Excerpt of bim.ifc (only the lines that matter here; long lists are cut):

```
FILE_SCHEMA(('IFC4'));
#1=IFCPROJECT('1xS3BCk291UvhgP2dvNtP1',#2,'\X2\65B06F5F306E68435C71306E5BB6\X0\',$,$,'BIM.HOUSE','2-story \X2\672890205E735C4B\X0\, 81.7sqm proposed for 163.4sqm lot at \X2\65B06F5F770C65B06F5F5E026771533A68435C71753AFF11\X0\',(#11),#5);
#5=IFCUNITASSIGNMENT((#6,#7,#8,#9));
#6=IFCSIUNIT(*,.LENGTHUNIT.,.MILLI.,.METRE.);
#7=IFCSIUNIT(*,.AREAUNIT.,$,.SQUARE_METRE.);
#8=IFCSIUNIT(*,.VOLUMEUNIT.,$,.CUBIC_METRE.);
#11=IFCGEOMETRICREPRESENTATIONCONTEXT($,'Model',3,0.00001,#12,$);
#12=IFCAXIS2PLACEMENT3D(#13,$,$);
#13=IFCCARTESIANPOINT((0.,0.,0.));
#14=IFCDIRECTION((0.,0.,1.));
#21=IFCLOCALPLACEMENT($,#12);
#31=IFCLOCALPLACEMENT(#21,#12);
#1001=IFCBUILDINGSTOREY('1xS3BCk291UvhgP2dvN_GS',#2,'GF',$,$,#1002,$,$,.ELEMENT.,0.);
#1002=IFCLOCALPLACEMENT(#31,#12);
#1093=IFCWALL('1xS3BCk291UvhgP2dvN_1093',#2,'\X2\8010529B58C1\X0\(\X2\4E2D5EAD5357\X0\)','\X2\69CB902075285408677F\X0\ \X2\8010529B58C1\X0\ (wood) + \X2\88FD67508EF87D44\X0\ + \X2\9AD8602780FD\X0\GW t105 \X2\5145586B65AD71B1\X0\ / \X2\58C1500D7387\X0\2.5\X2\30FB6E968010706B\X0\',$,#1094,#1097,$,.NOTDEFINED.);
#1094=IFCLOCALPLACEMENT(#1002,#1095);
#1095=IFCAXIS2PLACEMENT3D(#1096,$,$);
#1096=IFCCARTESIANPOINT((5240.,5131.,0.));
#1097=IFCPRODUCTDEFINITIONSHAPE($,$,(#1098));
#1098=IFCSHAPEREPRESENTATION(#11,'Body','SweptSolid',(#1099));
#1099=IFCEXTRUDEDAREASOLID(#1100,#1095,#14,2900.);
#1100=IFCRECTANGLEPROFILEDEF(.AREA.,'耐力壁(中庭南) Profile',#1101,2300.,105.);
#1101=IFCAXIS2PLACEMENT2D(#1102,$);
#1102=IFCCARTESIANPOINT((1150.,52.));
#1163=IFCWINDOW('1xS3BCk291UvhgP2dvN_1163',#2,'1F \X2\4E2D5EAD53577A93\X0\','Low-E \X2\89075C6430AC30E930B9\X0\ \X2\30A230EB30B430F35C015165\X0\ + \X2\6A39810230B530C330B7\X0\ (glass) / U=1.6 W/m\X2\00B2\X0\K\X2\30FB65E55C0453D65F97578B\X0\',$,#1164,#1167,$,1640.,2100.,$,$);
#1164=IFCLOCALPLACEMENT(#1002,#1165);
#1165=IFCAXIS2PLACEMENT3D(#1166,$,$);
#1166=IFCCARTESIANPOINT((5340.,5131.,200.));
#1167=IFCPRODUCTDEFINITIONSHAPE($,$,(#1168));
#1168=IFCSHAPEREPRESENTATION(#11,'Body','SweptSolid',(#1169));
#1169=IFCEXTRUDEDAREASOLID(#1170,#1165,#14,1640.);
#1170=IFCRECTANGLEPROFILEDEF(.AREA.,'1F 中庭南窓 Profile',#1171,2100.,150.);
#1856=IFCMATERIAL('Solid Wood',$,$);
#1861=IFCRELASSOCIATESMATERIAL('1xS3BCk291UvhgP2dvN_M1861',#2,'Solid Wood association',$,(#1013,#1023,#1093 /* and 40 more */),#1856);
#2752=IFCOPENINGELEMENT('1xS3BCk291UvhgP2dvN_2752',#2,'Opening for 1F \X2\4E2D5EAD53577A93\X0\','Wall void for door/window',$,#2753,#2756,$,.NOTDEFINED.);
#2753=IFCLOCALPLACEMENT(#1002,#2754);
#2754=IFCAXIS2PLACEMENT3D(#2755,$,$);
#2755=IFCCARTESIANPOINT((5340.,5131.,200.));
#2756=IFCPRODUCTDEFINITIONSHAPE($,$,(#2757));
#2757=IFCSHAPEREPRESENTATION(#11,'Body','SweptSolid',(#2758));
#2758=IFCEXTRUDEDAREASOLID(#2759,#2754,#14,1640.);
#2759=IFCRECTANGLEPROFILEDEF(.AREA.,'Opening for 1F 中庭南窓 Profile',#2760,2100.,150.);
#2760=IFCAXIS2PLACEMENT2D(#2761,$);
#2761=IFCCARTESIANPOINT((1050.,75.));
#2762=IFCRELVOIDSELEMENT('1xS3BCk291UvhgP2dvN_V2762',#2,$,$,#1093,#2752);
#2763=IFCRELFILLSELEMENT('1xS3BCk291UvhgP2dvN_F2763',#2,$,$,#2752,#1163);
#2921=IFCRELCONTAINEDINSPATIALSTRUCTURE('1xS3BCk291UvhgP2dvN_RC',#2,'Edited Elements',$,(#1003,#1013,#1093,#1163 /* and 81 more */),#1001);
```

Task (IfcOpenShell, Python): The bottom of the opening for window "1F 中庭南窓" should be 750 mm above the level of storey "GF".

```python
import numpy as np
import ifcopenshell
import ifcopenshell.api.geometry
import ifcopenshell.geom
import ifcopenshell.util.element
import ifcopenshell.util.placement
import ifcopenshell.util.shape
import ifcopenshell.util.unit

model = ifcopenshell.open("bim.ifc")
unit_scale = ifcopenshell.util.unit.calculate_unit_scale(model)

window = model.by_guid("1xS3BCk291UvhgP2dvN_1163")
opening = window.FillsVoids[0].RelatingOpeningElement
storey = ifcopenshell.util.element.get_container(window, ifc_class="IfcBuildingStorey")
level = ifcopenshell.util.placement.get_local_placement(storey.ObjectPlacement)[2, 3]

# The opening's origin need not be at the sill, so measure its lowest point.
shape = ifcopenshell.geom.create_shape(ifcopenshell.geom.settings(), opening)
bottom = ifcopenshell.util.shape.get_shape_bottom_elevation(shape, shape.geometry) / unit_scale
dz = level + 0.75 / unit_scale - bottom

shift = np.array([0.0, 0.0, dz])
# The window is not placed relative to its opening, so move both.
for product in (opening, window):
    matrix = ifcopenshell.util.placement.get_local_placement(product.ObjectPlacement)
    matrix[:3, 3] += shift
    ifcopenshell.api.geometry.edit_object_placement(model, product=product, matrix=matrix, is_si=False)

print(f"moved by {dz * unit_scale:+.3f} m")

model.write("bim_edited.ifc")
```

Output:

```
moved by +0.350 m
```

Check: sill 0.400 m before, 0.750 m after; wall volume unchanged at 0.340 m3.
